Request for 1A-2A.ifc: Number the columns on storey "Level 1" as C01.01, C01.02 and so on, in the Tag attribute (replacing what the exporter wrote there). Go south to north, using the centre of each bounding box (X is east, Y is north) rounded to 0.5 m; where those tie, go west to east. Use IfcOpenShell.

First a look at what the model holds.

```python
import ifcopenshell
import ifcopenshell.util.element
import ifcopenshell.util.placement

model = ifcopenshell.open("1A-2A.ifc")
print(model.schema)
storey = next(s for s in model.by_type("IfcBuildingStorey") if s.Name == "Level 1")
columns = [e for e in ifcopenshell.util.element.get_decomposition(storey) if e.is_a("IfcColumn")]
for e in sorted(columns, key=lambda e: e.id()):
    origin = ifcopenshell.util.placement.get_local_placement(e.ObjectPlacement)[:3, 3]
    print(e.id(), e.Tag, e.Name, origin.round(2) + 0.0, sep=" | ")
```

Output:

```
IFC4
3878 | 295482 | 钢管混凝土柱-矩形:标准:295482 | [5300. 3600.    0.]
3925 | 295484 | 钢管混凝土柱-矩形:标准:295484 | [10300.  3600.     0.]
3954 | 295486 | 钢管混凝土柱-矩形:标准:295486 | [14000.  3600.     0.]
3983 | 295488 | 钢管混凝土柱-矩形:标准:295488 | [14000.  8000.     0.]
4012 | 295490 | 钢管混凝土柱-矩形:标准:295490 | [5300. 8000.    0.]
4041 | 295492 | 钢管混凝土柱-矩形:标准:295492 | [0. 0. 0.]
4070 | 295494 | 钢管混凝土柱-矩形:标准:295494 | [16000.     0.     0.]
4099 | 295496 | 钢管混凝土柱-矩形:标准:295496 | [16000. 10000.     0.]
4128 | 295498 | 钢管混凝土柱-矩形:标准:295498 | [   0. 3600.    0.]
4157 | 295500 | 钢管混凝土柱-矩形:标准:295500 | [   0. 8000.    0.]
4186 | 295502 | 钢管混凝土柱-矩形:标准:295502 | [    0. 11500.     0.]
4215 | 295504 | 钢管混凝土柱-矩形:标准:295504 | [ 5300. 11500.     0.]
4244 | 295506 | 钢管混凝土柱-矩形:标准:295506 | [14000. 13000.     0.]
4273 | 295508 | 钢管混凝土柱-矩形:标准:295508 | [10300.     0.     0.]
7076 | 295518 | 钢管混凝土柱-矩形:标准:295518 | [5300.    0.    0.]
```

```python
import ifcopenshell
import ifcopenshell.geom
import ifcopenshell.util.element
import ifcopenshell.util.shape

model = ifcopenshell.open("1A-2A.ifc")
settings = ifcopenshell.geom.settings()
settings.set("use-world-coords", True)


def centre(element):
    shape = ifcopenshell.geom.create_shape(settings, element)
    return ifcopenshell.util.shape.get_bbox_centroid(shape.geometry)


storey = next(s for s in model.by_type("IfcBuildingStorey") if s.Name == "Level 1")
columns = [e for e in ifcopenshell.util.element.get_decomposition(storey) if e.is_a("IfcColumn")]

# Insertion points can sit at a corner or the storey origin, so sort by the geometry (in metres).
centres = {e: centre(e) for e in columns}
columns.sort(key=lambda e: (round(centres[e][1] / 0.5), centres[e][0]))

for i, e in enumerate(columns, start=1):
    number = f"C01.{i:02d}"
    e.Tag = number
    print(e.id(), number)

model.write("1A-2A-out.ifc")
```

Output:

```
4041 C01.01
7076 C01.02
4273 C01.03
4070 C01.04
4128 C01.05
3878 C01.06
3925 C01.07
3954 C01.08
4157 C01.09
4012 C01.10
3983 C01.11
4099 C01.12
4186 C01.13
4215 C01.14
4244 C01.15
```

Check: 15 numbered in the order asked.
